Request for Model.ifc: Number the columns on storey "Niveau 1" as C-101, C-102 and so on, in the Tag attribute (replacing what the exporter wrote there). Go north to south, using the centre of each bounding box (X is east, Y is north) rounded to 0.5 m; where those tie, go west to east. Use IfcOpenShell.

First a look at what the model holds.

```python
import ifcopenshell
import ifcopenshell.util.element
import ifcopenshell.util.placement

model = ifcopenshell.open("Model.ifc")
print(model.schema)
storey = next(s for s in model.by_type("IfcBuildingStorey") if s.Name == "Niveau 1")
columns = [e for e in ifcopenshell.util.element.get_decomposition(storey) if e.is_a("IfcColumn")]
for e in sorted(columns, key=lambda e: e.id()):
    origin = ifcopenshell.util.placement.get_local_placement(e.ObjectPlacement)[:3, 3]
    print(e.id(), e.Tag, e.Name, origin.round(2) + 0.0, sep=" | ")
```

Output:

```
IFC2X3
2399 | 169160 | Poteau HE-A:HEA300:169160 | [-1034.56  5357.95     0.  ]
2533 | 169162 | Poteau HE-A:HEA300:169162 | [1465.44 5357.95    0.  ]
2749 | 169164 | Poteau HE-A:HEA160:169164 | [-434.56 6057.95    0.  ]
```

```python
import ifcopenshell
import ifcopenshell.geom
import ifcopenshell.util.element
import ifcopenshell.util.shape

model = ifcopenshell.open("Model.ifc")
settings = ifcopenshell.geom.settings()
settings.set("use-world-coords", True)


def centre(element):
    shape = ifcopenshell.geom.create_shape(settings, element)
    return ifcopenshell.util.shape.get_bbox_centroid(shape.geometry)


storey = next(s for s in model.by_type("IfcBuildingStorey") if s.Name == "Niveau 1")
columns = [e for e in ifcopenshell.util.element.get_decomposition(storey) if e.is_a("IfcColumn")]

# Insertion points can sit at a corner or the storey origin, so sort by the geometry (in metres).
centres = {e: centre(e) for e in columns}
columns.sort(key=lambda e: (-round(centres[e][1] / 0.5), centres[e][0]))

for i, e in enumerate(columns, start=1):
    number = f"C-1{i:02d}"
    e.Tag = number
    print(e.id(), number)

model.write("Model-out.ifc")
```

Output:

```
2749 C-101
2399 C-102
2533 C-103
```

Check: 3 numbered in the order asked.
